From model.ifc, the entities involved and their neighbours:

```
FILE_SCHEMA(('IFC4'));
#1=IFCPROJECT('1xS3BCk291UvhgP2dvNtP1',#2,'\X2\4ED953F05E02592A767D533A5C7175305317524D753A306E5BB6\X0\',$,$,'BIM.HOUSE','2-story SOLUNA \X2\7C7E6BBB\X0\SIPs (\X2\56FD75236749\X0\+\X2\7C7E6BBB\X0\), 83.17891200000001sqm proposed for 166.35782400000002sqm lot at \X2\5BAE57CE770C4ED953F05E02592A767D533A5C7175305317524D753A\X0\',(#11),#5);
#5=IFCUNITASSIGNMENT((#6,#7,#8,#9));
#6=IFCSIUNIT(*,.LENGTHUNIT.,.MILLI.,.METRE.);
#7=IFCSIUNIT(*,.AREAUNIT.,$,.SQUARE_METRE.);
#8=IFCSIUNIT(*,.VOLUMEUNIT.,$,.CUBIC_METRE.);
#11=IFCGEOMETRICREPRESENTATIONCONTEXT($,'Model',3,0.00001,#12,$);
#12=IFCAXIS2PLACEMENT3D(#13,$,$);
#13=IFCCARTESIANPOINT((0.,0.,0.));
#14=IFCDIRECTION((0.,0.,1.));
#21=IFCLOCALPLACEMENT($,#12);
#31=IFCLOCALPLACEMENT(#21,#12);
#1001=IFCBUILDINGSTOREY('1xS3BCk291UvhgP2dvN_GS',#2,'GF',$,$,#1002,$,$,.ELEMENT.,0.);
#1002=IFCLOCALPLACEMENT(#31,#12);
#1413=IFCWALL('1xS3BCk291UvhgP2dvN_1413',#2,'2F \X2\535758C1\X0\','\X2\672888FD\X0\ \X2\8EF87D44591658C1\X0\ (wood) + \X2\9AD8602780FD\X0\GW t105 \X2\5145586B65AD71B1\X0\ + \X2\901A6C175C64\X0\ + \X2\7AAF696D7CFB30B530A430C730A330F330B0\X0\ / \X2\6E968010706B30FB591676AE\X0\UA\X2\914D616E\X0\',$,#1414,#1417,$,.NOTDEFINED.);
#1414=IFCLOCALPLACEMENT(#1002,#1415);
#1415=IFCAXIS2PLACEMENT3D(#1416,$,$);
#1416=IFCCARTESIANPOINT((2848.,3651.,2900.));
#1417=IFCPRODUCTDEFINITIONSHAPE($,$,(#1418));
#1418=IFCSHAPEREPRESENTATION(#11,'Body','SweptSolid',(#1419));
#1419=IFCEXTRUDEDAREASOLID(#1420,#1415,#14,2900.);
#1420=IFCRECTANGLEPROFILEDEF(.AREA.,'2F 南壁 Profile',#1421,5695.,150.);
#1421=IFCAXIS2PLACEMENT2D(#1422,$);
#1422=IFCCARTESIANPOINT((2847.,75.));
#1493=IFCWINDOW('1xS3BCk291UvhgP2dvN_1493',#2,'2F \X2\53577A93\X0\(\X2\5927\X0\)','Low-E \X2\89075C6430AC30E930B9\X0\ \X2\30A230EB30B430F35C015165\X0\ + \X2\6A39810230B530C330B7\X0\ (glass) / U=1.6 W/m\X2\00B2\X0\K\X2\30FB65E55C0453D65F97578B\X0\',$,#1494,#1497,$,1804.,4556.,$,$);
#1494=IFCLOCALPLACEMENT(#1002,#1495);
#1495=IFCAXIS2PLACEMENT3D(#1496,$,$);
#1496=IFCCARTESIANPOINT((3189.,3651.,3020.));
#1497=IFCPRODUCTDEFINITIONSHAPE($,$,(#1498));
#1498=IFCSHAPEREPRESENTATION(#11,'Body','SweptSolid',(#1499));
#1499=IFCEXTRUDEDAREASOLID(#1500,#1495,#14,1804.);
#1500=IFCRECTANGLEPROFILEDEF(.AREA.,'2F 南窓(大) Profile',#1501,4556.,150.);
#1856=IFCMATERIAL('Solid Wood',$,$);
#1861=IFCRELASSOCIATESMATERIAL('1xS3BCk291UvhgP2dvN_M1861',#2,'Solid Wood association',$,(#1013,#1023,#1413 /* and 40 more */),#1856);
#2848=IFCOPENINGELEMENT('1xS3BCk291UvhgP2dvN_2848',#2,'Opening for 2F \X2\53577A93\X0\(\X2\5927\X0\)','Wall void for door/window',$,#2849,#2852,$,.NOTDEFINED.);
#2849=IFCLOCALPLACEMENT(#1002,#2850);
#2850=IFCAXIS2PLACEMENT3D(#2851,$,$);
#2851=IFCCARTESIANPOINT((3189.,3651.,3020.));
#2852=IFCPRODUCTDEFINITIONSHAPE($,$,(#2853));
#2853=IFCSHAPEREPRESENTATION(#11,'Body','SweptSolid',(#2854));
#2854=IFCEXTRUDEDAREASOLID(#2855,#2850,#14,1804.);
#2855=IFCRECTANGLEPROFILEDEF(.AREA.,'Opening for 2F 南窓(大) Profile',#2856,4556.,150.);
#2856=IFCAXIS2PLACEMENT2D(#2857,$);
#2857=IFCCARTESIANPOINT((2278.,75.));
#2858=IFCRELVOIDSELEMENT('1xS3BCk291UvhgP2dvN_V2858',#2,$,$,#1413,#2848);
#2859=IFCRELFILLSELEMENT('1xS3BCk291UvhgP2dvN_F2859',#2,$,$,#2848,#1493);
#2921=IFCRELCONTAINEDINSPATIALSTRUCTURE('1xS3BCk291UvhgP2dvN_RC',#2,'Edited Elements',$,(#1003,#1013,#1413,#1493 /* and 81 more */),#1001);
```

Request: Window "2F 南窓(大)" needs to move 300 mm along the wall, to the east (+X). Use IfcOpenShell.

```python
import ifcopenshell
import ifcopenshell.api.geometry
import ifcopenshell.util.placement

model = ifcopenshell.open("model.ifc")

window = model.by_guid("1xS3BCk291UvhgP2dvN_1493")
opening = window.FillsVoids[0].RelatingOpeningElement
wall = opening.VoidsElements[0].RelatingBuildingElement

wall_matrix = ifcopenshell.util.placement.get_local_placement(wall.ObjectPlacement)
shift = wall_matrix[:3, 0] * 300.0
before = ifcopenshell.util.placement.get_local_placement(window.ObjectPlacement)[:3, 3].copy()

# The window is not placed relative to its opening, so move both.
for product in (opening, window):
    matrix = ifcopenshell.util.placement.get_local_placement(product.ObjectPlacement)
    matrix[:3, 3] += shift
    ifcopenshell.api.geometry.edit_object_placement(model, product=product, matrix=matrix, is_si=False)

after = ifcopenshell.util.placement.get_local_placement(window.ObjectPlacement)[:3, 3]
print("window moved by", (after - before).round(3) + 0.0)

model.write("model-out.ifc")
```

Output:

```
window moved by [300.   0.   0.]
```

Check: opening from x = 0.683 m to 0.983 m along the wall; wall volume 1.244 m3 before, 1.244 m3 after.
